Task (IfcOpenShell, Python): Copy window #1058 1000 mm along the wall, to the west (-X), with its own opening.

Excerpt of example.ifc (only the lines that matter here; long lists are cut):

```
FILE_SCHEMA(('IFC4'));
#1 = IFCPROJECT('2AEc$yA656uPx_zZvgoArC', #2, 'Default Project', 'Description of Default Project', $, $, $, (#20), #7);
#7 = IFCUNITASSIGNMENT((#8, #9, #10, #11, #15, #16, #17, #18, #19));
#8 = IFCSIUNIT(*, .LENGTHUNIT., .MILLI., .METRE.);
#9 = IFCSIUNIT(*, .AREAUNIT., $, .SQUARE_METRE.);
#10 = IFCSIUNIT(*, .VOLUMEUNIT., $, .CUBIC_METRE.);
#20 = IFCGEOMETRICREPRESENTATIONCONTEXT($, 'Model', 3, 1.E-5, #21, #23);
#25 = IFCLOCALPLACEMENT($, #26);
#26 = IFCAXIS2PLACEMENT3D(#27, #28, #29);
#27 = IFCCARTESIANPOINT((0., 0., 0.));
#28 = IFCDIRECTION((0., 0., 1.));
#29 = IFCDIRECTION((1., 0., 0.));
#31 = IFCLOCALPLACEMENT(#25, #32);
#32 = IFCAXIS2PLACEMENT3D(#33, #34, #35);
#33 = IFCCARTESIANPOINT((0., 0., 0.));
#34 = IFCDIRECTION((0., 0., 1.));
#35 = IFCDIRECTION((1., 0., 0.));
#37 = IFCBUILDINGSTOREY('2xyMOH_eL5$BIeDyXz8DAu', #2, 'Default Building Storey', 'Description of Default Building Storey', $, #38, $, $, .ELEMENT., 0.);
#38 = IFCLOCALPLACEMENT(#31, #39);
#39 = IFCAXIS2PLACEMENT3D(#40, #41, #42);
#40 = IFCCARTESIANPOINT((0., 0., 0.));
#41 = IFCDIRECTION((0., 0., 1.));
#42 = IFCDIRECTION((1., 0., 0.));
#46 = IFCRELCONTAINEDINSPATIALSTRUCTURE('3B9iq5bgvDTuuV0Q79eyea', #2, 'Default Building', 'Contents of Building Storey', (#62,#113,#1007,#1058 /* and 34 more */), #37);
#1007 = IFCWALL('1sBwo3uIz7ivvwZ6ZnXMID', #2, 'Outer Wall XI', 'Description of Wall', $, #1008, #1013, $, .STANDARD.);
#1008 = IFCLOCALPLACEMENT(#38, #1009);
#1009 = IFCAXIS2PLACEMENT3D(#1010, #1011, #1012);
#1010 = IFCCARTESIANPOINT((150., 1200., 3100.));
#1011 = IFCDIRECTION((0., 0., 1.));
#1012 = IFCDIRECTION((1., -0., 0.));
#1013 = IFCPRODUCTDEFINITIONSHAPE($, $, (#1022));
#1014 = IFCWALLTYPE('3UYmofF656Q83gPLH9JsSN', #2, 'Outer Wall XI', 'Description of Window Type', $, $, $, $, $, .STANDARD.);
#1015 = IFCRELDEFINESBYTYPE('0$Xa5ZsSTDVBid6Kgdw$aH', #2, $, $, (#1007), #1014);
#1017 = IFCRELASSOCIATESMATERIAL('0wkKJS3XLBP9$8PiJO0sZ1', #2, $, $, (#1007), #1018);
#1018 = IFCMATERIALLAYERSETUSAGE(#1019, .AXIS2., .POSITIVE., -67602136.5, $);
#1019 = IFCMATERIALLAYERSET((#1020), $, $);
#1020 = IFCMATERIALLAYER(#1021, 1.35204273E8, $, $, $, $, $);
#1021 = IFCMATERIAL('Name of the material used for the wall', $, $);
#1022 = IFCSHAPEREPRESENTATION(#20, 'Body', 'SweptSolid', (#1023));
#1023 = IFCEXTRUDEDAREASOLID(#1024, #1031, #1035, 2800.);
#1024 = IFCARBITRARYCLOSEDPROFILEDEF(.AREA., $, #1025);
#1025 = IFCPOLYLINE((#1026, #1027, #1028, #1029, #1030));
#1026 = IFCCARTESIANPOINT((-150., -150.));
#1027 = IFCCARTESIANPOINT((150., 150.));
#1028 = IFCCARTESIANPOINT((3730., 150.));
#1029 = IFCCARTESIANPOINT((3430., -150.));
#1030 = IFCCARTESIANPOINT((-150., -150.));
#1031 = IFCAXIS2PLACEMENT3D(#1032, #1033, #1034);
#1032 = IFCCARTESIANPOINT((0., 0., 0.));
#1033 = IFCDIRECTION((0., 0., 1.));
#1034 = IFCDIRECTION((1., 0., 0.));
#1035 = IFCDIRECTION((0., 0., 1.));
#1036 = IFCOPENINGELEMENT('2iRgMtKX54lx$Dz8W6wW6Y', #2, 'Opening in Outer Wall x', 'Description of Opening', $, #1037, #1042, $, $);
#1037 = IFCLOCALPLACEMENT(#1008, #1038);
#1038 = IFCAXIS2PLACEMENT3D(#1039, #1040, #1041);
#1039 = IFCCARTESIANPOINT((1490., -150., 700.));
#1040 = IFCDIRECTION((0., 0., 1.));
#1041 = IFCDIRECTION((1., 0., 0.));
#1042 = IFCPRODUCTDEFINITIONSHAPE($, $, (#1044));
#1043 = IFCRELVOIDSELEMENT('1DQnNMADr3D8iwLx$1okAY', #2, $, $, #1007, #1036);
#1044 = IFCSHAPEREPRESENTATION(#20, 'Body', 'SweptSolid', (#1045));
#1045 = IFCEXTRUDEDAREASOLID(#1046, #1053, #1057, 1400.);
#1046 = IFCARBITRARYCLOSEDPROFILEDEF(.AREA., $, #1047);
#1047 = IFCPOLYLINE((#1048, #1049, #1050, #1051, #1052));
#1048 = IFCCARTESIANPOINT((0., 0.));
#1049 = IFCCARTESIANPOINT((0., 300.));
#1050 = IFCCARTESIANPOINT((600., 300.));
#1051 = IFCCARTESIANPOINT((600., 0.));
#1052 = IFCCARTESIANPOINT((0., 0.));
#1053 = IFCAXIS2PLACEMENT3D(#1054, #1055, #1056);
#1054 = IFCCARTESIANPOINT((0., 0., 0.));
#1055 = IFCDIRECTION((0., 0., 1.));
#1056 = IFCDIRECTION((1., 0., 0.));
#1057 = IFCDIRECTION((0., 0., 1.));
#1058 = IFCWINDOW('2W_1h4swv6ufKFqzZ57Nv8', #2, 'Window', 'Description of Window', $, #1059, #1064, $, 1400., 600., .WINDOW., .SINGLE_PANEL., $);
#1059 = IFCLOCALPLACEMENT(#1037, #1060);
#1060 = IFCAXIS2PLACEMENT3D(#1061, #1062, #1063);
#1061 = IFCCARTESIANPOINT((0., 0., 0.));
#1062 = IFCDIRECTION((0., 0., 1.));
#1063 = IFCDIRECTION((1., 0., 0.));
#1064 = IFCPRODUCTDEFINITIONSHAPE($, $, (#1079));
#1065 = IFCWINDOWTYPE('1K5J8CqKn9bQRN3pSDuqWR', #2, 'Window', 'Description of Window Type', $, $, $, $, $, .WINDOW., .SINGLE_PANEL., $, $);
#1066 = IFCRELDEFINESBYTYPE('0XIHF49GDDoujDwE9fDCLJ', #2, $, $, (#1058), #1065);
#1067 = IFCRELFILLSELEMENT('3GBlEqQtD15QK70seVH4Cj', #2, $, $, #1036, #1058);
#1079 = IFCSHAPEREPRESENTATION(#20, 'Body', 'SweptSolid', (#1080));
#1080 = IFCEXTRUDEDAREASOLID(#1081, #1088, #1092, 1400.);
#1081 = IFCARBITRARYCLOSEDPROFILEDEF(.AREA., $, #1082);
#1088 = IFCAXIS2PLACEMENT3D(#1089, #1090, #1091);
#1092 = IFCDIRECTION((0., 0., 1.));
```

```python
import ifcopenshell
import ifcopenshell.api.feature
import ifcopenshell.api.geometry
import ifcopenshell.api.root
import ifcopenshell.geom
import ifcopenshell.util.element
import ifcopenshell.util.placement
import ifcopenshell.util.shape

model = ifcopenshell.open("example.ifc")
settings = ifcopenshell.geom.settings()


def volume(element):
    """Net volume in cubic metres, openings subtracted."""
    shape = ifcopenshell.geom.create_shape(settings, element)
    return ifcopenshell.util.shape.get_volume(shape.geometry)


def reuse_history(source, copy):
    """copy_class also copies each property set's owner history, people and application; keep the originals."""
    for rel in copy.IsDefinedBy:
        if rel.is_a("IfcRelDefinesByProperties") and (history := rel.RelatingPropertyDefinition.OwnerHistory):
            rel.RelatingPropertyDefinition.OwnerHistory = source.OwnerHistory
            ifcopenshell.util.element.remove_deep2(model, history)


window = model.by_id(1058)
opening = window.FillsVoids[0].RelatingOpeningElement
wall = opening.VoidsElements[0].RelatingBuildingElement
before = volume(wall)
shift = ifcopenshell.util.placement.get_local_placement(wall.ObjectPlacement)[:3, 0] * -1000.0

# copy_class copies the void relationship, type, container and properties, but no geometry.
new_opening = ifcopenshell.api.root.copy_class(model, product=opening)
new_opening.Representation = ifcopenshell.util.element.copy_deep(
    model, opening.Representation, exclude=["IfcGeometricRepresentationContext", "IfcRepresentationMap"]
)
new_window = ifcopenshell.api.root.copy_class(model, product=window)
new_window.Representation = ifcopenshell.util.element.copy_deep(
    model, window.Representation, exclude=["IfcGeometricRepresentationContext", "IfcRepresentationMap"]
)
reuse_history(window, new_window)
ifcopenshell.api.feature.add_filling(model, opening=new_opening, element=new_window)

for old, new in ((opening, new_opening), (window, new_window)):
    matrix = ifcopenshell.util.placement.get_local_placement(old.ObjectPlacement)
    matrix[:3, 3] += shift
    ifcopenshell.api.geometry.edit_object_placement(model, product=new, matrix=matrix, is_si=False)

after = volume(wall)

print(f"wall volume {before:.3f} -> {after:.3f} m3")

model.write("example_rev.ifc")
```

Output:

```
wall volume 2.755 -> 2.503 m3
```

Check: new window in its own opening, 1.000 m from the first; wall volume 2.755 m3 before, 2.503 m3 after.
